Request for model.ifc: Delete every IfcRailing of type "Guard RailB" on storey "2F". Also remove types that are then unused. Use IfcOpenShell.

First a look at what the model holds.

```python
import ifcopenshell
import ifcopenshell.util.element

model = ifcopenshell.open("model.ifc")
print(model.schema)
storey = next(s for s in model.by_type("IfcBuildingStorey") if s.Name == "2F")
railings = [e for e in ifcopenshell.util.element.get_decomposition(storey) if e.is_a("IfcRailing")]
seen = {}
for e in railings:
    element_type = ifcopenshell.util.element.get_type(e)
    name = element_type.Name if element_type not in (None, e) else None
    seen[name] = seen.get(name, 0) + 1
for name, count in sorted(seen.items(), key=str):
    print(count, "x", name)
```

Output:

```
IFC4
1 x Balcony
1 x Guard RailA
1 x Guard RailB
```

```python
import ifcopenshell
import ifcopenshell.api.root
import ifcopenshell.util.element

model = ifcopenshell.open("model.ifc")

storey = next(s for s in model.by_type("IfcBuildingStorey") if s.Name == "2F")
railings = [e for e in ifcopenshell.util.element.get_decomposition(storey) if e.is_a("IfcRailing")]
targets = [e for e in railings if (t := ifcopenshell.util.element.get_type(e)) not in (None, e) and t.Name == "Guard RailB"]
types = {ifcopenshell.util.element.get_type(e) for e in targets} - {None, *targets}

for e in targets:
    ifcopenshell.api.root.remove_product(model, product=e)
print(len(targets), "removed")

unused = [t for t in types if not ifcopenshell.util.element.get_types(t)]
for t in unused:
    ifcopenshell.api.root.remove_product(model, product=t)
print(len(unused), "unused types removed")

model.write("model_edited.ifc")
```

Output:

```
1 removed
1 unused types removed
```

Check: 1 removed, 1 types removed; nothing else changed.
